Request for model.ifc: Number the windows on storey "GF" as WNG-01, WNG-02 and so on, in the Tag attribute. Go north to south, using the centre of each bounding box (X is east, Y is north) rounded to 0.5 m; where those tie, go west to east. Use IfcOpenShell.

First a look at what the model holds.

```python
import ifcopenshell
import ifcopenshell.util.element
import ifcopenshell.util.placement

model = ifcopenshell.open("model.ifc")
print(model.schema)
storey = next(s for s in model.by_type("IfcBuildingStorey") if s.Name == "GF")
windows = [e for e in ifcopenshell.util.element.get_decomposition(storey) if e.is_a("IfcWindow")]
for e in sorted(windows, key=lambda e: e.id()):
    origin = ifcopenshell.util.placement.get_local_placement(e.ObjectPlacement)[:3, 3]
    print(e.id(), e.Tag, e.Name, origin.round(2) + 0.0, sep=" | ")
```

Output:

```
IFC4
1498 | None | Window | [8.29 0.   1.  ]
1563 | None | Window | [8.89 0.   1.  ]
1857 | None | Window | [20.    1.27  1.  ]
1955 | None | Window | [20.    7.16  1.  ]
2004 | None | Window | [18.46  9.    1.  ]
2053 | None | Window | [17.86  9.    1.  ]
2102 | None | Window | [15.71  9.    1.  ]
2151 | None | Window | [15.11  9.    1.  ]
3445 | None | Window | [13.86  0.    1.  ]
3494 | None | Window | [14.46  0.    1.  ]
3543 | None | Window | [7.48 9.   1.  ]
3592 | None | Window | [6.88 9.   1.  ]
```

```python
import ifcopenshell
import ifcopenshell.geom
import ifcopenshell.util.element
import ifcopenshell.util.shape

model = ifcopenshell.open("model.ifc")
settings = ifcopenshell.geom.settings()
settings.set("use-world-coords", True)


def centre(element):
    shape = ifcopenshell.geom.create_shape(settings, element)
    return ifcopenshell.util.shape.get_bbox_centroid(shape.geometry)


storey = next(s for s in model.by_type("IfcBuildingStorey") if s.Name == "GF")
windows = [e for e in ifcopenshell.util.element.get_decomposition(storey) if e.is_a("IfcWindow")]

# Insertion points can sit at a corner or the storey origin, so sort by the geometry (in metres).
centres = {e: centre(e) for e in windows}
windows.sort(key=lambda e: (-round(centres[e][1] / 0.5), centres[e][0]))

for i, e in enumerate(windows, start=1):
    number = f"WNG-{i:02d}"
    e.Tag = number
    print(e.id(), number)

model.write("model-out.ifc")
```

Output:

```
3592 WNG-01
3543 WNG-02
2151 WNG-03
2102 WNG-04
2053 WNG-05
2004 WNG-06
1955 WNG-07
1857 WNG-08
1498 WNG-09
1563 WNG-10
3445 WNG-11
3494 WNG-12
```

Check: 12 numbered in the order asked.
